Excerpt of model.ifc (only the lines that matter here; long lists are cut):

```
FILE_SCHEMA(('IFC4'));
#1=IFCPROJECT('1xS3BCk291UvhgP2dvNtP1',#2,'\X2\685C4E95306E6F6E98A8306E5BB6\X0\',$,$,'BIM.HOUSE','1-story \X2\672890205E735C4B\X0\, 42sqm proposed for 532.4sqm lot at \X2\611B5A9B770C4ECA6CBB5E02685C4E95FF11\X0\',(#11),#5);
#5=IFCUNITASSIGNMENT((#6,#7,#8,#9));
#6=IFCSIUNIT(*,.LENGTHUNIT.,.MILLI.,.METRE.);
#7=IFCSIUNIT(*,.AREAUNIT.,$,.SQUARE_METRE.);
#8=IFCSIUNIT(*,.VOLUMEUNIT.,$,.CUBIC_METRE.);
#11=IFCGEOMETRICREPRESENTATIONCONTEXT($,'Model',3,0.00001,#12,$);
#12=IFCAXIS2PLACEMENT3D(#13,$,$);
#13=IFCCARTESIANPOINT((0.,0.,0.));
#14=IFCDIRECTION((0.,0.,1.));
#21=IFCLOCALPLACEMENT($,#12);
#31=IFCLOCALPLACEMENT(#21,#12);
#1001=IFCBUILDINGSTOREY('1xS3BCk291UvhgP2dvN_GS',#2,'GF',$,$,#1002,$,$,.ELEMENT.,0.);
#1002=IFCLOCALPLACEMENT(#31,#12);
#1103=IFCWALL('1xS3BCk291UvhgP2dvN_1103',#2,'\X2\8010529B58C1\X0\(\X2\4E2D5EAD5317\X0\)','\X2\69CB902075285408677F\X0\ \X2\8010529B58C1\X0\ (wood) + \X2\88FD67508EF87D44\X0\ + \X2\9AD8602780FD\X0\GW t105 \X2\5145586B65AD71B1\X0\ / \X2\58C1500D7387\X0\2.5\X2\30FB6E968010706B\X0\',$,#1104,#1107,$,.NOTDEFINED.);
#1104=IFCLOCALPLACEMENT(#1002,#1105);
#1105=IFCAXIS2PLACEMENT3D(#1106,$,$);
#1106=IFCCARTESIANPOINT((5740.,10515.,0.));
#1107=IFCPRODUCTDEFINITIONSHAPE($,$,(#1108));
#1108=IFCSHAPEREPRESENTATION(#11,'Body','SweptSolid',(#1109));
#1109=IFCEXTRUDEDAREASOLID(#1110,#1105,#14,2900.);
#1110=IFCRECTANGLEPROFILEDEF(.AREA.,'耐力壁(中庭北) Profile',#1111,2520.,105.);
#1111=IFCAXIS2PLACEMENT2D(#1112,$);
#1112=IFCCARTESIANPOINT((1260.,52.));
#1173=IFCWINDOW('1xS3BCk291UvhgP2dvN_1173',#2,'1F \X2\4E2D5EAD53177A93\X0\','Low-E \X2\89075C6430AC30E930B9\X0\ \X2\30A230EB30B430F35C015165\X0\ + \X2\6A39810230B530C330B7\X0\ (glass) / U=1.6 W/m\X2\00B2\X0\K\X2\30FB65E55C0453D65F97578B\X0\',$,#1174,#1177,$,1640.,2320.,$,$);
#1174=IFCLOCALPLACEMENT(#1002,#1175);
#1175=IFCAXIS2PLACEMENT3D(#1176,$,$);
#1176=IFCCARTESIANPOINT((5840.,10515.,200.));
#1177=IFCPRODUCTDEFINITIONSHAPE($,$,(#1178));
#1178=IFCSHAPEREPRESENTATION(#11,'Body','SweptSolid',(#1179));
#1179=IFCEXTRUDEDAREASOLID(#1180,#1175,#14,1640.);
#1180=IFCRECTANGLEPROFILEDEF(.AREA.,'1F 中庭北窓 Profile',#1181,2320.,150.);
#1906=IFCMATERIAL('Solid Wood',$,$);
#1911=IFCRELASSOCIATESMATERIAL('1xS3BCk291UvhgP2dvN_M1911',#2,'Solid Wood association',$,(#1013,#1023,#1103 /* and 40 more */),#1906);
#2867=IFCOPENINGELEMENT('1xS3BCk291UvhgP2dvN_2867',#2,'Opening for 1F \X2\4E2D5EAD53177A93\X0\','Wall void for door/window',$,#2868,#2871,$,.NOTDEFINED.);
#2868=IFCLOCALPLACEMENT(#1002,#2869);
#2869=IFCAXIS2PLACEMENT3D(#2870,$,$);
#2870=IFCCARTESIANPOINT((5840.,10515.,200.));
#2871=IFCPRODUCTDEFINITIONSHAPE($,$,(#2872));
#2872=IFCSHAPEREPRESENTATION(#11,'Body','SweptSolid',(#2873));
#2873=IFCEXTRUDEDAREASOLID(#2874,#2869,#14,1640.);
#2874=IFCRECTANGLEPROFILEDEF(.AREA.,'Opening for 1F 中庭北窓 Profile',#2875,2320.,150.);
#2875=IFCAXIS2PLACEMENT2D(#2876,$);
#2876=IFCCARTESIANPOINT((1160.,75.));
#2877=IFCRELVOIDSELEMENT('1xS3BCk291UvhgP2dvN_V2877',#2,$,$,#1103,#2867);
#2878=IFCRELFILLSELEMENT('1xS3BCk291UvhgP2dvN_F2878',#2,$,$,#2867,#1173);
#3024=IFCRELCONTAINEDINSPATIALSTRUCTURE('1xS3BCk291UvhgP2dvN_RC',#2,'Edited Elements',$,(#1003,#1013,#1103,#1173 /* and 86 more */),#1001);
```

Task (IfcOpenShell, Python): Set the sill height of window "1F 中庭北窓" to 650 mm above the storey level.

```python
import numpy as np
import ifcopenshell
import ifcopenshell.api.geometry
import ifcopenshell.geom
import ifcopenshell.util.element
import ifcopenshell.util.placement
import ifcopenshell.util.shape
import ifcopenshell.util.unit

model = ifcopenshell.open("model.ifc")
unit_scale = ifcopenshell.util.unit.calculate_unit_scale(model)

window = model.by_guid("1xS3BCk291UvhgP2dvN_1173")
opening = window.FillsVoids[0].RelatingOpeningElement
storey = ifcopenshell.util.element.get_container(window, ifc_class="IfcBuildingStorey")
level = ifcopenshell.util.placement.get_local_placement(storey.ObjectPlacement)[2, 3]

# The opening's origin need not be at the sill, so measure its lowest point.
shape = ifcopenshell.geom.create_shape(ifcopenshell.geom.settings(), opening)
bottom = ifcopenshell.util.shape.get_shape_bottom_elevation(shape, shape.geometry) / unit_scale
dz = level + 0.65 / unit_scale - bottom

shift = np.array([0.0, 0.0, dz])
# The window is not placed relative to its opening, so move both.
for product in (opening, window):
    matrix = ifcopenshell.util.placement.get_local_placement(product.ObjectPlacement)
    matrix[:3, 3] += shift
    ifcopenshell.api.geometry.edit_object_placement(model, product=product, matrix=matrix, is_si=False)

print(f"moved by {dz * unit_scale:+.3f} m")

model.write("model_rev.ifc")
```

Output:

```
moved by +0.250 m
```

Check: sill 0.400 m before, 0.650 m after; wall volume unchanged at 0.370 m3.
